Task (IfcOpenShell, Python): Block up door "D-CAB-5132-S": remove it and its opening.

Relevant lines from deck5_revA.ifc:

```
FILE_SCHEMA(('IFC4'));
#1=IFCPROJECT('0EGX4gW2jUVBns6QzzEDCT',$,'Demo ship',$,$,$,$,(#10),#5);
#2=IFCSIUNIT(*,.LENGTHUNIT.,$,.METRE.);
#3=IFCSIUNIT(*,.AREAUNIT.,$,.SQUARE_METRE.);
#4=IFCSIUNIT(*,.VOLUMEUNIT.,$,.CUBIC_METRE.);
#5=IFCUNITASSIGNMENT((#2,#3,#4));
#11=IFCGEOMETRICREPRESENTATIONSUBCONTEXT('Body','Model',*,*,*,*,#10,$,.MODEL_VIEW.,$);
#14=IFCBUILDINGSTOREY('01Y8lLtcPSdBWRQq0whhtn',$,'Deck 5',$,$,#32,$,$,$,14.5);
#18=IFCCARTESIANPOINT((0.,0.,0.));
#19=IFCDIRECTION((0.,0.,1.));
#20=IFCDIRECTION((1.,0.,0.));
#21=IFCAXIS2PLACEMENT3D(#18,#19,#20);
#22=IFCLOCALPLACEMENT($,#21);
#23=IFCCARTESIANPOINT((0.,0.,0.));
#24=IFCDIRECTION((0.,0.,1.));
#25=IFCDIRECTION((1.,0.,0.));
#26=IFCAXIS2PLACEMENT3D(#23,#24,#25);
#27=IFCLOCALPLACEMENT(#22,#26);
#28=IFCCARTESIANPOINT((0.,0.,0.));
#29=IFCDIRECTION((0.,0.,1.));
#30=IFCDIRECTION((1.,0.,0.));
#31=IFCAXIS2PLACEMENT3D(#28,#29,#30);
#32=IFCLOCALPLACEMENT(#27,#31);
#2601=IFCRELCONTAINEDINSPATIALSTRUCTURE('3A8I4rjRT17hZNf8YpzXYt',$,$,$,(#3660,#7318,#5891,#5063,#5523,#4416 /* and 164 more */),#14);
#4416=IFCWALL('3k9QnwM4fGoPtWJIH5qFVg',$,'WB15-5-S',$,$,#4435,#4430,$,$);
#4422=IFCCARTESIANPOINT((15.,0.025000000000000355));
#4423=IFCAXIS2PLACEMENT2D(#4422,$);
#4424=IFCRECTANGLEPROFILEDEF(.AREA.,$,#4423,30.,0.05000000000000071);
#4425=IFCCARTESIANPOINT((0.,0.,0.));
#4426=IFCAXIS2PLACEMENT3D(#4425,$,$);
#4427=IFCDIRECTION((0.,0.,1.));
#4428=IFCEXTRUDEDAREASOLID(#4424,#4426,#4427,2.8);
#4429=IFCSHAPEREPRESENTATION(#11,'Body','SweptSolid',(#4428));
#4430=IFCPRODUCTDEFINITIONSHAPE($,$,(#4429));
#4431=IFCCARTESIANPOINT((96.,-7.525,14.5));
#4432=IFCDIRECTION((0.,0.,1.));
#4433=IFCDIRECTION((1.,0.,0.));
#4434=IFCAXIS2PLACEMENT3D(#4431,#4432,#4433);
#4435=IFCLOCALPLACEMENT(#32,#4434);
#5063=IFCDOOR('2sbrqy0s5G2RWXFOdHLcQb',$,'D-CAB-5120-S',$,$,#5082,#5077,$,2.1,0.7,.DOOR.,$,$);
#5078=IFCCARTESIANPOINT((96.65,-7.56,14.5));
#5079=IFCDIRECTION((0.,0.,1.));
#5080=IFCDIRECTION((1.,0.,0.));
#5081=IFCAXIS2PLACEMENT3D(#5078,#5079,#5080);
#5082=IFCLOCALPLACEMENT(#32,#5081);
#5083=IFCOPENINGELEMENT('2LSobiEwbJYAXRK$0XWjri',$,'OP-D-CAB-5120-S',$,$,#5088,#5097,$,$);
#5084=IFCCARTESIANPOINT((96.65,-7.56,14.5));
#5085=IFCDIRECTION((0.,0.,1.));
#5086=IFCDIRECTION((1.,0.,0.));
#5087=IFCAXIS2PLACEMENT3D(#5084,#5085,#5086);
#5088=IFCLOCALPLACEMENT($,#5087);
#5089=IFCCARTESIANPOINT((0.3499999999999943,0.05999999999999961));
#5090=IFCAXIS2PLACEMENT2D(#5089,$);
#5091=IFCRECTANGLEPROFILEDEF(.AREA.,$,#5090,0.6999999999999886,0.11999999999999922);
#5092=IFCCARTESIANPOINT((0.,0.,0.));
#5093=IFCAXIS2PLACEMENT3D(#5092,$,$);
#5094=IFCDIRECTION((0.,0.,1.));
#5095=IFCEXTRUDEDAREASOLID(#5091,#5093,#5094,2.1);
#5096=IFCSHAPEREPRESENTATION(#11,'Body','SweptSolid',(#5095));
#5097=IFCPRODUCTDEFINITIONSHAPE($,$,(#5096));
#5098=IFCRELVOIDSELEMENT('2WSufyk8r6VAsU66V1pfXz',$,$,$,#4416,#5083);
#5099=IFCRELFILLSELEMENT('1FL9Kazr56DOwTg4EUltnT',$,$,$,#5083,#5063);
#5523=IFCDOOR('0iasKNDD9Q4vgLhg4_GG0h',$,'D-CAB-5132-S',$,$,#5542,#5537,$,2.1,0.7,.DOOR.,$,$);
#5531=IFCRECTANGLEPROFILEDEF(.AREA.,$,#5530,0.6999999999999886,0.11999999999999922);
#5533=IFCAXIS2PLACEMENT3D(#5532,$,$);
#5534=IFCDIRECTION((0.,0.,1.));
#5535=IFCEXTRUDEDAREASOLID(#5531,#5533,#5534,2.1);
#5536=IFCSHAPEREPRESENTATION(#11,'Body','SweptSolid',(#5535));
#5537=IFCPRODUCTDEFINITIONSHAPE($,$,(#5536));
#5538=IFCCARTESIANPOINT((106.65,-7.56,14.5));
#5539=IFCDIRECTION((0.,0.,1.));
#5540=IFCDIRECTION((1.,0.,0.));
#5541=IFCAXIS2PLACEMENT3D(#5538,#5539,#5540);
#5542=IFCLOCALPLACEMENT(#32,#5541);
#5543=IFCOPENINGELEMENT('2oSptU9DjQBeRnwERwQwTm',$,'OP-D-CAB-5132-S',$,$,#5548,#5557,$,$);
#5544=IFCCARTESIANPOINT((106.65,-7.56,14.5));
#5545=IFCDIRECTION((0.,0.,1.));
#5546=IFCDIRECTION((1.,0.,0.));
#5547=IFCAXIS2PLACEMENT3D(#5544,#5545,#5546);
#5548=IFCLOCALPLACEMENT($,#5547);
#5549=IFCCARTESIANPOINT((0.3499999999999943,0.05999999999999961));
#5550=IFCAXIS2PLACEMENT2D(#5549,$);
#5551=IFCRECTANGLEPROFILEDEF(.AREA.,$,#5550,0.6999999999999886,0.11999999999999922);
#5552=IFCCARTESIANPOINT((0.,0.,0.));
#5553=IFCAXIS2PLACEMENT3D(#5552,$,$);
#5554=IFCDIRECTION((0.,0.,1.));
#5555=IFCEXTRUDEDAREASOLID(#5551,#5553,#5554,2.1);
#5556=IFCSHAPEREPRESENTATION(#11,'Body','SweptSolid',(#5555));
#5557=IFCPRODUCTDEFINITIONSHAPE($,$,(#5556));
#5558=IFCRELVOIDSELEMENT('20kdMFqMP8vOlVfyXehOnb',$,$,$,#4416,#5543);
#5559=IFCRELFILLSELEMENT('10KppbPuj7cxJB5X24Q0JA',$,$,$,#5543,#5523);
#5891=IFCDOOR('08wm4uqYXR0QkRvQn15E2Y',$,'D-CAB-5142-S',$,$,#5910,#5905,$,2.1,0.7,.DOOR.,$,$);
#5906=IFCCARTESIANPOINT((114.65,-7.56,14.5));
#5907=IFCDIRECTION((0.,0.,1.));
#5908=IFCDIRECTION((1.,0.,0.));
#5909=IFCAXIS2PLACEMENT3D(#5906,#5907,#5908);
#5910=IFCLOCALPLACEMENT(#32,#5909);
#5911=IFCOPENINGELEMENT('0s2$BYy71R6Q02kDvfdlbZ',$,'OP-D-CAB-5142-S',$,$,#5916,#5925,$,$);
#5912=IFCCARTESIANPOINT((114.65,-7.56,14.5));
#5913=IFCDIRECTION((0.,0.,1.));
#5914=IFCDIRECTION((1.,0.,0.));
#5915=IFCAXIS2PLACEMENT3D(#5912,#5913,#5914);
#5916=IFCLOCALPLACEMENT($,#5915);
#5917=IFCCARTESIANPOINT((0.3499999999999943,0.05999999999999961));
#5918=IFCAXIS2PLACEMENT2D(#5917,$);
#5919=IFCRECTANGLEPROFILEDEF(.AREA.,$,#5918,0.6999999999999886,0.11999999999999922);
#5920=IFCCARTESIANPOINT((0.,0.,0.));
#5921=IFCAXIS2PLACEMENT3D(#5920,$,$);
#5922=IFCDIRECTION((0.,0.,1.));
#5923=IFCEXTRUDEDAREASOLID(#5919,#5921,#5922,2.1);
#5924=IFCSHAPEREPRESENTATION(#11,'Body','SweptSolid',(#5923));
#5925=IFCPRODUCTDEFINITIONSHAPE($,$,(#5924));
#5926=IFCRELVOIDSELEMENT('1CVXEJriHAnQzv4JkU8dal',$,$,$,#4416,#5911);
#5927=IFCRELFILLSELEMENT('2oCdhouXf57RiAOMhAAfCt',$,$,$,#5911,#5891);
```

```python
import ifcopenshell
import ifcopenshell.api.feature
import ifcopenshell.api.root
import ifcopenshell.geom
import ifcopenshell.util.shape

model = ifcopenshell.open("deck5_revA.ifc")
settings = ifcopenshell.geom.settings()


def volume(element):
    """Net volume in cubic metres, openings subtracted."""
    shape = ifcopenshell.geom.create_shape(settings, element)
    return ifcopenshell.util.shape.get_volume(shape.geometry)


door = model.by_guid("0iasKNDD9Q4vgLhg4_GG0h")
opening = door.FillsVoids[0].RelatingOpeningElement
wall = opening.VoidsElements[0].RelatingBuildingElement
before = volume(wall)

ifcopenshell.api.root.remove_product(model, product=door)
ifcopenshell.api.feature.remove_feature(model, feature=opening)

after = volume(wall)

print(f"wall volume {before:.3f} -> {after:.3f} m3")

model.write("deck5_revA_edited.ifc")
```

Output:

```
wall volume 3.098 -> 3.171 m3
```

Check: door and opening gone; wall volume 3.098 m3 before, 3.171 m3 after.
